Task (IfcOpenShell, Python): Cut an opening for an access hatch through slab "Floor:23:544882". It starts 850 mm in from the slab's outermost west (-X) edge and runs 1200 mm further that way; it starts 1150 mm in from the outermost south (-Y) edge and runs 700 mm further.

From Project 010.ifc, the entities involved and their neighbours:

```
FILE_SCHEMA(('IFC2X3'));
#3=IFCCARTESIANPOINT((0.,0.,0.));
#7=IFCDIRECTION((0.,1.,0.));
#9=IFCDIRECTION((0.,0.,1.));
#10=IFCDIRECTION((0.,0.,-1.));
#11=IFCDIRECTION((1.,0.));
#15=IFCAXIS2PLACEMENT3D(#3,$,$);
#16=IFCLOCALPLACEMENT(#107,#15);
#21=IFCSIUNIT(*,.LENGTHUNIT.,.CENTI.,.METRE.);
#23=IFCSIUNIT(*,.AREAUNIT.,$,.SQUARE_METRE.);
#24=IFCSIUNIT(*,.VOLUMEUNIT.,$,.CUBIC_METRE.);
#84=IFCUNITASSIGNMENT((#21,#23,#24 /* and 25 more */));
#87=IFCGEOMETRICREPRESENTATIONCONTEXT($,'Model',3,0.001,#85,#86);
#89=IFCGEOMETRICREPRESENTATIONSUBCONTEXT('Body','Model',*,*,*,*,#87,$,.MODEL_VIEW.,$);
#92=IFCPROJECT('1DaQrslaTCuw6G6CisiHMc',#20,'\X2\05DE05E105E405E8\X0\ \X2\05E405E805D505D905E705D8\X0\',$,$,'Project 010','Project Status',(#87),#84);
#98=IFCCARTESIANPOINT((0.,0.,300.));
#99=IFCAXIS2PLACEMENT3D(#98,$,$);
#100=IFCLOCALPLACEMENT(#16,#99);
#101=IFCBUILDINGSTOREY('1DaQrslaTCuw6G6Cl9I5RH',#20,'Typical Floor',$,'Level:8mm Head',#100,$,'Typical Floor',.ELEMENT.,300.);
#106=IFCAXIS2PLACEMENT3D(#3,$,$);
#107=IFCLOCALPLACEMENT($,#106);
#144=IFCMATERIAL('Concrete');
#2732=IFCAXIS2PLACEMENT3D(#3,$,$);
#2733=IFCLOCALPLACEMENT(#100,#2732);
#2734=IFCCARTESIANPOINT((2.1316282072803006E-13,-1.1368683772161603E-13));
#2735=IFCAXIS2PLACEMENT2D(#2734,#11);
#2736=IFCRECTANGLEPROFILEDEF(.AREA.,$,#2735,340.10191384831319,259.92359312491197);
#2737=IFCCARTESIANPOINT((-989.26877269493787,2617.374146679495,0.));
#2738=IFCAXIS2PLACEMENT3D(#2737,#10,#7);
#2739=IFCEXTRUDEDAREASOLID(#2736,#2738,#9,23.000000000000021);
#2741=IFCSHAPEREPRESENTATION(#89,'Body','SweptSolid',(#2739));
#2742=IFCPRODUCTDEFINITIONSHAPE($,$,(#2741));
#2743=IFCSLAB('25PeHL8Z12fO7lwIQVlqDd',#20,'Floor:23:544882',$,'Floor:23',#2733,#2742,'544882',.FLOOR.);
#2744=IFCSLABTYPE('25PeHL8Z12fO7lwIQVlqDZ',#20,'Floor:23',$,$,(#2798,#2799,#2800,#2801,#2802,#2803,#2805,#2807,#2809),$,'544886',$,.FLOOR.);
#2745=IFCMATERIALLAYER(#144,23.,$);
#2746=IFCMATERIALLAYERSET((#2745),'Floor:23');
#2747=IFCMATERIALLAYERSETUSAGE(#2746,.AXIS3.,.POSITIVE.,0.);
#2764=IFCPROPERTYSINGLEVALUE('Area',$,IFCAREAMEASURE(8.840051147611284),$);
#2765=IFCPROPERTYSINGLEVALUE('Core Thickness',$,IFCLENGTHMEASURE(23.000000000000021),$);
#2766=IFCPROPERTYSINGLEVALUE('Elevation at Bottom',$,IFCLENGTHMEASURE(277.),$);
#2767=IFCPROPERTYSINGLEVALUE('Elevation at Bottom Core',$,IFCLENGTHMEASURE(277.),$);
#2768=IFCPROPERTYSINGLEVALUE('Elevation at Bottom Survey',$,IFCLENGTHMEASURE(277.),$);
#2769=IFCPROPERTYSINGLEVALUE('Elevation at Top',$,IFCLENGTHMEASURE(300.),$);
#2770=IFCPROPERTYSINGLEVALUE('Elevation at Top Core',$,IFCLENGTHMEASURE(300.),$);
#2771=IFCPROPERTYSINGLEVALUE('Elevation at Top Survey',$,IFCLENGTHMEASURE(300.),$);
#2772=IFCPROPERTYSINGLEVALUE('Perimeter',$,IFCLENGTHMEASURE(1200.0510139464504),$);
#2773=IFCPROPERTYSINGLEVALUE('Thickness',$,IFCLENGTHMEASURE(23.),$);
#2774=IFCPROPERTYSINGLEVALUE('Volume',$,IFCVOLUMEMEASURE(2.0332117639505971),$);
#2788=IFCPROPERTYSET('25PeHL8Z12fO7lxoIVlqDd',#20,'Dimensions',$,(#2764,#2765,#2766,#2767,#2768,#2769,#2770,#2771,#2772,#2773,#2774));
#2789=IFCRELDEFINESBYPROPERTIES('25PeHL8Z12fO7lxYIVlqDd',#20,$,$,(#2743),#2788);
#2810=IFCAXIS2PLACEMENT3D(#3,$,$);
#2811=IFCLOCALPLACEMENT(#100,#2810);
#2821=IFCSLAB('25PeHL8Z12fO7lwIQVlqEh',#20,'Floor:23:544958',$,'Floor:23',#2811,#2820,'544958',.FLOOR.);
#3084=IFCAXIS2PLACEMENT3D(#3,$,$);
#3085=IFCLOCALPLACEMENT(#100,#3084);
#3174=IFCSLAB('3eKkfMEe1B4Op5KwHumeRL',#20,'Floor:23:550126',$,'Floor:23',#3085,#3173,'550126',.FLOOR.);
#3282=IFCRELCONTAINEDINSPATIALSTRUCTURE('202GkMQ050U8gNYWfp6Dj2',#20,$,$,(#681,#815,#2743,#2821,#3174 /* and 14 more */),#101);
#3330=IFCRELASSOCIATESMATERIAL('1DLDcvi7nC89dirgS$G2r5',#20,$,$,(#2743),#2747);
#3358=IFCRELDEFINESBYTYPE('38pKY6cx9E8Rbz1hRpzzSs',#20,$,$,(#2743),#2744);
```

```python
import numpy as np
import ifcopenshell
import ifcopenshell.api.feature
import ifcopenshell.api.geometry
import ifcopenshell.api.pset
import ifcopenshell.api.root
import ifcopenshell.geom
import ifcopenshell.util.element
import ifcopenshell.util.placement
import ifcopenshell.util.representation
import ifcopenshell.util.shape
import ifcopenshell.util.unit

model = ifcopenshell.open("Project 010.ifc")
unit_scale = ifcopenshell.util.unit.calculate_unit_scale(model)
area_scale = ifcopenshell.util.unit.calculate_unit_scale(model, "AREAUNIT")
volume_scale = ifcopenshell.util.unit.calculate_unit_scale(model, "VOLUMEUNIT")
settings = ifcopenshell.geom.settings()


def volume(element):
    """Net volume in cubic metres, openings subtracted."""
    shape = ifcopenshell.geom.create_shape(settings, element)
    return ifcopenshell.util.shape.get_volume(shape.geometry)


slab = model.by_id(2743)
before = volume(slab)

# Extent in the slab's own axes, in metres. The edges named are its -X and -Y sides.
slab_shape = ifcopenshell.geom.create_shape(settings, slab)
vertices = ifcopenshell.util.shape.get_vertices(slab_shape.geometry)
x_min, y_min, bottom = vertices.min(axis=0)
top = vertices[:, 2].max()

opening = ifcopenshell.api.root.create_entity(model, ifc_class="IfcOpeningElement", name="Access hatch opening")
context = ifcopenshell.util.representation.get_context(model, "Model", "Body", "MODEL_VIEW")
width, depth = 1.2, 0.7
outline = [(0.0, 0.0), (width, 0.0), (width, depth), (0.0, depth), (0.0, 0.0)]
# Overshoot both faces by 50 mm so the cut is clean.
shape = ifcopenshell.api.geometry.add_slab_representation(
    model, context=context, depth=top - bottom + 0.1, polyline=outline
)
ifcopenshell.api.geometry.assign_representation(model, product=opening, representation=shape)

matrix = ifcopenshell.util.placement.get_local_placement(slab.ObjectPlacement)
matrix[:, 3] = matrix @ np.append(np.array([x_min + 0.85, y_min + 1.15, bottom - 0.05]) / unit_scale, 1.0)
ifcopenshell.api.geometry.edit_object_placement(model, product=opening, matrix=matrix, is_si=False)
ifcopenshell.api.feature.add_feature(model, feature=opening, element=slab)

after = volume(slab)

# Update the slab's stored quantities.
pset = model.by_id(ifcopenshell.util.element.get_pset(slab, "Dimensions", should_inherit=False)["id"])
ifcopenshell.api.pset.edit_pset(model, pset=pset, properties={
    "Area": model.create_entity("IfcAreaMeasure", after / (top - bottom) / area_scale),
    "Volume": model.create_entity("IfcVolumeMeasure", after / volume_scale),
})

print(f"slab volume {before:.3f} -> {after:.3f} m3")

model.write("Project 010_v2.ifc")
```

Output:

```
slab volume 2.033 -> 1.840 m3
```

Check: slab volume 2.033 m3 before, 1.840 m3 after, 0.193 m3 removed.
